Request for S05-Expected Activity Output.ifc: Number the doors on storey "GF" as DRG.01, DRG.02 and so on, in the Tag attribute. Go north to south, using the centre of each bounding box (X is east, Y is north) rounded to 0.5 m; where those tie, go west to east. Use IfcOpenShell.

First a look at what the model holds.

```python
import ifcopenshell
import ifcopenshell.util.element
import ifcopenshell.util.placement

model = ifcopenshell.open("S05-Expected Activity Output.ifc")
print(model.schema)
storey = next(s for s in model.by_type("IfcBuildingStorey") if s.Name == "GF")
doors = [e for e in ifcopenshell.util.element.get_decomposition(storey) if e.is_a("IfcDoor")]
for e in sorted(doors, key=lambda e: e.id()):
    origin = ifcopenshell.util.placement.get_local_placement(e.ObjectPlacement)[:3, 3]
    print(e.id(), e.Tag, e.Name, origin.round(2) + 0.0, sep=" | ")
```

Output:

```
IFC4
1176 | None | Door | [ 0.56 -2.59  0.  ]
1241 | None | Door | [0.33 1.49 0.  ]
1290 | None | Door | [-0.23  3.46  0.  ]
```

```python
import ifcopenshell
import ifcopenshell.geom
import ifcopenshell.util.element
import ifcopenshell.util.shape

model = ifcopenshell.open("S05-Expected Activity Output.ifc")
settings = ifcopenshell.geom.settings()
settings.set("use-world-coords", True)


def centre(element):
    shape = ifcopenshell.geom.create_shape(settings, element)
    return ifcopenshell.util.shape.get_bbox_centroid(shape.geometry)


storey = next(s for s in model.by_type("IfcBuildingStorey") if s.Name == "GF")
doors = [e for e in ifcopenshell.util.element.get_decomposition(storey) if e.is_a("IfcDoor")]

# Insertion points can sit at a corner or the storey origin, so sort by the geometry (in metres).
centres = {e: centre(e) for e in doors}
doors.sort(key=lambda e: (-round(centres[e][1] / 0.5), centres[e][0]))

for i, e in enumerate(doors, start=1):
    number = f"DRG.{i:02d}"
    e.Tag = number
    print(e.id(), number)

model.write("S05-Expected Activity Output_v2.ifc")
```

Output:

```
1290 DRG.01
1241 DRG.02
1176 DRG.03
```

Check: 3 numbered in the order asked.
